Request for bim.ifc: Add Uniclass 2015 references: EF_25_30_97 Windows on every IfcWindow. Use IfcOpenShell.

First a look at what the model holds.

```python
import ifcopenshell

model = ifcopenshell.open("bim.ifc")
print(model.schema)
print("classifications:", [c.Name for c in model.by_type("IfcClassification")])
for ifc_class in ("IfcDoor", "IfcRoof", "IfcStair", "IfcWall", "IfcWindow"):
    print(ifc_class, len(model.by_type(ifc_class)))
```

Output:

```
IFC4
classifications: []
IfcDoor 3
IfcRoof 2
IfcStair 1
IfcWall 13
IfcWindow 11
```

```python
import ifcopenshell
import ifcopenshell.api.classification

model = ifcopenshell.open("bim.ifc")

system = ifcopenshell.api.classification.add_classification(model, classification="Uniclass 2015")

codes = {
    "IfcWindow": ("EF_25_30_97", "Windows"),
}
for ifc_class, (code, name) in codes.items():
    products = model.by_type(ifc_class)
    ifcopenshell.api.classification.add_reference(
        model, products=products, classification=system, identification=code, name=name
    )
    print(code, len(products))

model.write("bim_updated.ifc")
```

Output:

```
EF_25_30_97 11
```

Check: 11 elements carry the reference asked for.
